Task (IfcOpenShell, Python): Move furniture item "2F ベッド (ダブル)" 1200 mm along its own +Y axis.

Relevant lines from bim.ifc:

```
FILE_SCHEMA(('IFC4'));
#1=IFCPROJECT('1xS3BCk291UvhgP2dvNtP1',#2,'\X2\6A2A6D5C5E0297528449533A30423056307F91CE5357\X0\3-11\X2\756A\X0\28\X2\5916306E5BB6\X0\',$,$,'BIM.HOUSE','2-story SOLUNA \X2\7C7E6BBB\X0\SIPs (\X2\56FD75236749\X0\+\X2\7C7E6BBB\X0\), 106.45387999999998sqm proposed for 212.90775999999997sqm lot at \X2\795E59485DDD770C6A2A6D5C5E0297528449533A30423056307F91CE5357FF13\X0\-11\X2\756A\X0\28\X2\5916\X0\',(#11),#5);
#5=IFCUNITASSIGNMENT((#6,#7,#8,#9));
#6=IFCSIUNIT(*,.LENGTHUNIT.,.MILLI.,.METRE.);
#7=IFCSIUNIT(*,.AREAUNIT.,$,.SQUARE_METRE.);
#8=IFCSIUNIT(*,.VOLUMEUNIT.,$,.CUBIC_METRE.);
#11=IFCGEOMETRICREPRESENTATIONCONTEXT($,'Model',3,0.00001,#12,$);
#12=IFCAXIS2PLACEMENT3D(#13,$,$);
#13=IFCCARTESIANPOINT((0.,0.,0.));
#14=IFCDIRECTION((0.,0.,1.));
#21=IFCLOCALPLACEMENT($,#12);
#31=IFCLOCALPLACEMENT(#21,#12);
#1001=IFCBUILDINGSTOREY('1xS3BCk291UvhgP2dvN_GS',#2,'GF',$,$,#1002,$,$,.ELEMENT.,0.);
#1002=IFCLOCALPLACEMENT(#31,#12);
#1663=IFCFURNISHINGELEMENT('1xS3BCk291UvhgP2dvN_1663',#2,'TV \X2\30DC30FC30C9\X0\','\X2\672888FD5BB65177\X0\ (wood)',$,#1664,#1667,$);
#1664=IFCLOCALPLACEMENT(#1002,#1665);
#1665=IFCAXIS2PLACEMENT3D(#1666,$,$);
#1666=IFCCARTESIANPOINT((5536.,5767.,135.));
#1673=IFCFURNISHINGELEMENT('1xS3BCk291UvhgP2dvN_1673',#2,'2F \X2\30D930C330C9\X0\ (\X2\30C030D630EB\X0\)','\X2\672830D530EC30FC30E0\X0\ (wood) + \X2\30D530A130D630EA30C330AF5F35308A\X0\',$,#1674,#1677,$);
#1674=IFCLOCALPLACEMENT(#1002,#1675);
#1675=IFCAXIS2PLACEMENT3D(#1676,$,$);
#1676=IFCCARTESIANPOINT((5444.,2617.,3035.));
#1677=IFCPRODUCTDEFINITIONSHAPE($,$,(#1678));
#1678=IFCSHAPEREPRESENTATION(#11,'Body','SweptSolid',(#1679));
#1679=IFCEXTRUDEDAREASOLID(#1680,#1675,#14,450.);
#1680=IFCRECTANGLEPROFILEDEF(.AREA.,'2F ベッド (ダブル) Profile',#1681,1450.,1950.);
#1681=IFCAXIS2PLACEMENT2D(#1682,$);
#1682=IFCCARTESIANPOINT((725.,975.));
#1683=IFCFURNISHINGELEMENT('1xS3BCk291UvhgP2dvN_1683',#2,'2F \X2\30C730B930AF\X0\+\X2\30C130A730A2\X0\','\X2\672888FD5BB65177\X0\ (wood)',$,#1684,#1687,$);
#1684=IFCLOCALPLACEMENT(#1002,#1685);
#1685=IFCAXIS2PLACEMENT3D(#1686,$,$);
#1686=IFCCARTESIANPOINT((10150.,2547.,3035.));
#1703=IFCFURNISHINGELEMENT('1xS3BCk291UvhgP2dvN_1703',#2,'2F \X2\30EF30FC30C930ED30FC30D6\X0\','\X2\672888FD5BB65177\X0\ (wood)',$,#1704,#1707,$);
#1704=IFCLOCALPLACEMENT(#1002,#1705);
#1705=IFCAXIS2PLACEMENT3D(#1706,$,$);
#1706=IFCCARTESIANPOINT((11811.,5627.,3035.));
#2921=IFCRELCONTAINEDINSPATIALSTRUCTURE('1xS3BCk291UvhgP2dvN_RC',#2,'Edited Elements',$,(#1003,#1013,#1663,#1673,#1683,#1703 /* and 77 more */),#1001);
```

```python
import ifcopenshell
import ifcopenshell.api.geometry
import ifcopenshell.util.placement

model = ifcopenshell.open("bim.ifc")

item = model.by_guid("1xS3BCk291UvhgP2dvN_1673")
matrix = ifcopenshell.util.placement.get_local_placement(item.ObjectPlacement)
matrix[:3, 3] += matrix[:3, 1] * 1200.0
ifcopenshell.api.geometry.edit_object_placement(model, product=item, matrix=matrix, is_si=False)

print(ifcopenshell.util.placement.get_local_placement(item.ObjectPlacement).round(3) + 0.0)

model.write("bim_edited.ifc")
```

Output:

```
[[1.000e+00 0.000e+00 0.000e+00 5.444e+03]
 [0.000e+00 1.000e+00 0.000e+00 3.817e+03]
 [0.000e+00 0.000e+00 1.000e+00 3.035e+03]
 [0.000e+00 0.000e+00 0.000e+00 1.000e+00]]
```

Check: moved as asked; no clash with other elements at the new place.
